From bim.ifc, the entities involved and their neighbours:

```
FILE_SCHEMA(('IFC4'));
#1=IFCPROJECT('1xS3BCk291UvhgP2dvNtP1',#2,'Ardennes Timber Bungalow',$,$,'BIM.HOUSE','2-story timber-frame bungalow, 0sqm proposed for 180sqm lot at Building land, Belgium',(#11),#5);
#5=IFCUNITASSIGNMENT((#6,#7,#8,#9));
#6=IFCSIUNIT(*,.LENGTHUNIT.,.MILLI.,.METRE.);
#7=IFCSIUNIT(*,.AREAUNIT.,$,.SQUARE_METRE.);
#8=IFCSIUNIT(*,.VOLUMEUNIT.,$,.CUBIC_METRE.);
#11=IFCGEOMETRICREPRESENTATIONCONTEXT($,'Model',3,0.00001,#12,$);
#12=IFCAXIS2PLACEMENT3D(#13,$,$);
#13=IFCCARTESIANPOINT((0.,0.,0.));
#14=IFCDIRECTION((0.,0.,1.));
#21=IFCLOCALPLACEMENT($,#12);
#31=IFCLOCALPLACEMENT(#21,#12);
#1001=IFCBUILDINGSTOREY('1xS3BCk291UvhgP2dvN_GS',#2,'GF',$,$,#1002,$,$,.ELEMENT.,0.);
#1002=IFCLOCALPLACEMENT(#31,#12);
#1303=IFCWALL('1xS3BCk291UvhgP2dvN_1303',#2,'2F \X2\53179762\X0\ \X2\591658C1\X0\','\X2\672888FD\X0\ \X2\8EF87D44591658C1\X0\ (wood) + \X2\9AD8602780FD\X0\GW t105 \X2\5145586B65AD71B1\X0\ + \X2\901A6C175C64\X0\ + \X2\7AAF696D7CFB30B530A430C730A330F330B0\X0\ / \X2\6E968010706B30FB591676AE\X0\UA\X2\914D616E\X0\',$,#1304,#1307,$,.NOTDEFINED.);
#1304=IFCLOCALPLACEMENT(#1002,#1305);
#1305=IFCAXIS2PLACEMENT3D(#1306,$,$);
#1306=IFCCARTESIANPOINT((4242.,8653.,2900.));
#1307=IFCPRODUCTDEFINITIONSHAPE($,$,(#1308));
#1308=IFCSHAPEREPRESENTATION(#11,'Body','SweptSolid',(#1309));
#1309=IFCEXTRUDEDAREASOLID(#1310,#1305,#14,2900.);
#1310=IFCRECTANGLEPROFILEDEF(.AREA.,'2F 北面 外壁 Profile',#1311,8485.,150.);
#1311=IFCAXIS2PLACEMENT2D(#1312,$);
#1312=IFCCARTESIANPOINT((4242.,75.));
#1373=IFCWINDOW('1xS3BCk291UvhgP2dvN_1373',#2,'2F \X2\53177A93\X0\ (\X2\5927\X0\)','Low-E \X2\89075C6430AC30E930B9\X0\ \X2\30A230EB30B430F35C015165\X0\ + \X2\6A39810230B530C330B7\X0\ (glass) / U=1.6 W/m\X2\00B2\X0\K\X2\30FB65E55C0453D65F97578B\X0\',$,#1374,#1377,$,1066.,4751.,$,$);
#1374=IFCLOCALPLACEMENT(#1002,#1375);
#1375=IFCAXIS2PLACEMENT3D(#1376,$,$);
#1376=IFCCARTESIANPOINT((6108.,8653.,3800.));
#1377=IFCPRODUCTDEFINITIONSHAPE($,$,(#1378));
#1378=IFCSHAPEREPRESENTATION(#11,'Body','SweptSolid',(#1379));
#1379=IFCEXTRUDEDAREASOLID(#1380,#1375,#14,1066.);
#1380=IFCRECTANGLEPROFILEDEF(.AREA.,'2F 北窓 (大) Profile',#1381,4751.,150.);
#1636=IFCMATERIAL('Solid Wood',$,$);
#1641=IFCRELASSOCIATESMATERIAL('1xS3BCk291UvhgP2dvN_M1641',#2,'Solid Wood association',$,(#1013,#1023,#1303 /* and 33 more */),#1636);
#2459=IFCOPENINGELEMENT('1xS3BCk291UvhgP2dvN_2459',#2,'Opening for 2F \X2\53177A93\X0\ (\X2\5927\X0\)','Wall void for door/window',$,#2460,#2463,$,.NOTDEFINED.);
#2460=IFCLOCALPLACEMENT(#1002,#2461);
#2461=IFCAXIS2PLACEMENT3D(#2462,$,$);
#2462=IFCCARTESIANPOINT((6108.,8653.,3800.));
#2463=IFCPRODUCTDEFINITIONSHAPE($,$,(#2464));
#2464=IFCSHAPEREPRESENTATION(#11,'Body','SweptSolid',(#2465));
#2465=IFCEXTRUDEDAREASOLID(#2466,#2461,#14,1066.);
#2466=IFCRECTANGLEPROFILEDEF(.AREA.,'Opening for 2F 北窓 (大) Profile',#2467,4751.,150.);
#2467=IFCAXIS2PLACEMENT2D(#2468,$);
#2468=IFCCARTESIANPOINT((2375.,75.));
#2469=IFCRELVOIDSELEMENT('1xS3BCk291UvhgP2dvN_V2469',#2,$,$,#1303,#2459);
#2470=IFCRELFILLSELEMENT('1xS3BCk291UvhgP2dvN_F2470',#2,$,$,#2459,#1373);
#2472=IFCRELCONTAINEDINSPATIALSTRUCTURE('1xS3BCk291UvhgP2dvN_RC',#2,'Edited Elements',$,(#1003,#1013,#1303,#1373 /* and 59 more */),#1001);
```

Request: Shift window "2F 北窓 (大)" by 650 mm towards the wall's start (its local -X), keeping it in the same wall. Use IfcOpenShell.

```python
import ifcopenshell
import ifcopenshell.api.geometry
import ifcopenshell.util.placement

model = ifcopenshell.open("bim.ifc")

window = model.by_guid("1xS3BCk291UvhgP2dvN_1373")
opening = window.FillsVoids[0].RelatingOpeningElement
wall = opening.VoidsElements[0].RelatingBuildingElement

wall_matrix = ifcopenshell.util.placement.get_local_placement(wall.ObjectPlacement)
shift = wall_matrix[:3, 0] * -650.0
before = ifcopenshell.util.placement.get_local_placement(window.ObjectPlacement)[:3, 3].copy()

# The window is not placed relative to its opening, so move both.
for product in (opening, window):
    matrix = ifcopenshell.util.placement.get_local_placement(product.ObjectPlacement)
    matrix[:3, 3] += shift
    ifcopenshell.api.geometry.edit_object_placement(model, product=product, matrix=matrix, is_si=False)

after = ifcopenshell.util.placement.get_local_placement(window.ObjectPlacement)[:3, 3]
print("window moved by", (after - before).round(3) + 0.0)

model.write("bim_rev.ifc")
```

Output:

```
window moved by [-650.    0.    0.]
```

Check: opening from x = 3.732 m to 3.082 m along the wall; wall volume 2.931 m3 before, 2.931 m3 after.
